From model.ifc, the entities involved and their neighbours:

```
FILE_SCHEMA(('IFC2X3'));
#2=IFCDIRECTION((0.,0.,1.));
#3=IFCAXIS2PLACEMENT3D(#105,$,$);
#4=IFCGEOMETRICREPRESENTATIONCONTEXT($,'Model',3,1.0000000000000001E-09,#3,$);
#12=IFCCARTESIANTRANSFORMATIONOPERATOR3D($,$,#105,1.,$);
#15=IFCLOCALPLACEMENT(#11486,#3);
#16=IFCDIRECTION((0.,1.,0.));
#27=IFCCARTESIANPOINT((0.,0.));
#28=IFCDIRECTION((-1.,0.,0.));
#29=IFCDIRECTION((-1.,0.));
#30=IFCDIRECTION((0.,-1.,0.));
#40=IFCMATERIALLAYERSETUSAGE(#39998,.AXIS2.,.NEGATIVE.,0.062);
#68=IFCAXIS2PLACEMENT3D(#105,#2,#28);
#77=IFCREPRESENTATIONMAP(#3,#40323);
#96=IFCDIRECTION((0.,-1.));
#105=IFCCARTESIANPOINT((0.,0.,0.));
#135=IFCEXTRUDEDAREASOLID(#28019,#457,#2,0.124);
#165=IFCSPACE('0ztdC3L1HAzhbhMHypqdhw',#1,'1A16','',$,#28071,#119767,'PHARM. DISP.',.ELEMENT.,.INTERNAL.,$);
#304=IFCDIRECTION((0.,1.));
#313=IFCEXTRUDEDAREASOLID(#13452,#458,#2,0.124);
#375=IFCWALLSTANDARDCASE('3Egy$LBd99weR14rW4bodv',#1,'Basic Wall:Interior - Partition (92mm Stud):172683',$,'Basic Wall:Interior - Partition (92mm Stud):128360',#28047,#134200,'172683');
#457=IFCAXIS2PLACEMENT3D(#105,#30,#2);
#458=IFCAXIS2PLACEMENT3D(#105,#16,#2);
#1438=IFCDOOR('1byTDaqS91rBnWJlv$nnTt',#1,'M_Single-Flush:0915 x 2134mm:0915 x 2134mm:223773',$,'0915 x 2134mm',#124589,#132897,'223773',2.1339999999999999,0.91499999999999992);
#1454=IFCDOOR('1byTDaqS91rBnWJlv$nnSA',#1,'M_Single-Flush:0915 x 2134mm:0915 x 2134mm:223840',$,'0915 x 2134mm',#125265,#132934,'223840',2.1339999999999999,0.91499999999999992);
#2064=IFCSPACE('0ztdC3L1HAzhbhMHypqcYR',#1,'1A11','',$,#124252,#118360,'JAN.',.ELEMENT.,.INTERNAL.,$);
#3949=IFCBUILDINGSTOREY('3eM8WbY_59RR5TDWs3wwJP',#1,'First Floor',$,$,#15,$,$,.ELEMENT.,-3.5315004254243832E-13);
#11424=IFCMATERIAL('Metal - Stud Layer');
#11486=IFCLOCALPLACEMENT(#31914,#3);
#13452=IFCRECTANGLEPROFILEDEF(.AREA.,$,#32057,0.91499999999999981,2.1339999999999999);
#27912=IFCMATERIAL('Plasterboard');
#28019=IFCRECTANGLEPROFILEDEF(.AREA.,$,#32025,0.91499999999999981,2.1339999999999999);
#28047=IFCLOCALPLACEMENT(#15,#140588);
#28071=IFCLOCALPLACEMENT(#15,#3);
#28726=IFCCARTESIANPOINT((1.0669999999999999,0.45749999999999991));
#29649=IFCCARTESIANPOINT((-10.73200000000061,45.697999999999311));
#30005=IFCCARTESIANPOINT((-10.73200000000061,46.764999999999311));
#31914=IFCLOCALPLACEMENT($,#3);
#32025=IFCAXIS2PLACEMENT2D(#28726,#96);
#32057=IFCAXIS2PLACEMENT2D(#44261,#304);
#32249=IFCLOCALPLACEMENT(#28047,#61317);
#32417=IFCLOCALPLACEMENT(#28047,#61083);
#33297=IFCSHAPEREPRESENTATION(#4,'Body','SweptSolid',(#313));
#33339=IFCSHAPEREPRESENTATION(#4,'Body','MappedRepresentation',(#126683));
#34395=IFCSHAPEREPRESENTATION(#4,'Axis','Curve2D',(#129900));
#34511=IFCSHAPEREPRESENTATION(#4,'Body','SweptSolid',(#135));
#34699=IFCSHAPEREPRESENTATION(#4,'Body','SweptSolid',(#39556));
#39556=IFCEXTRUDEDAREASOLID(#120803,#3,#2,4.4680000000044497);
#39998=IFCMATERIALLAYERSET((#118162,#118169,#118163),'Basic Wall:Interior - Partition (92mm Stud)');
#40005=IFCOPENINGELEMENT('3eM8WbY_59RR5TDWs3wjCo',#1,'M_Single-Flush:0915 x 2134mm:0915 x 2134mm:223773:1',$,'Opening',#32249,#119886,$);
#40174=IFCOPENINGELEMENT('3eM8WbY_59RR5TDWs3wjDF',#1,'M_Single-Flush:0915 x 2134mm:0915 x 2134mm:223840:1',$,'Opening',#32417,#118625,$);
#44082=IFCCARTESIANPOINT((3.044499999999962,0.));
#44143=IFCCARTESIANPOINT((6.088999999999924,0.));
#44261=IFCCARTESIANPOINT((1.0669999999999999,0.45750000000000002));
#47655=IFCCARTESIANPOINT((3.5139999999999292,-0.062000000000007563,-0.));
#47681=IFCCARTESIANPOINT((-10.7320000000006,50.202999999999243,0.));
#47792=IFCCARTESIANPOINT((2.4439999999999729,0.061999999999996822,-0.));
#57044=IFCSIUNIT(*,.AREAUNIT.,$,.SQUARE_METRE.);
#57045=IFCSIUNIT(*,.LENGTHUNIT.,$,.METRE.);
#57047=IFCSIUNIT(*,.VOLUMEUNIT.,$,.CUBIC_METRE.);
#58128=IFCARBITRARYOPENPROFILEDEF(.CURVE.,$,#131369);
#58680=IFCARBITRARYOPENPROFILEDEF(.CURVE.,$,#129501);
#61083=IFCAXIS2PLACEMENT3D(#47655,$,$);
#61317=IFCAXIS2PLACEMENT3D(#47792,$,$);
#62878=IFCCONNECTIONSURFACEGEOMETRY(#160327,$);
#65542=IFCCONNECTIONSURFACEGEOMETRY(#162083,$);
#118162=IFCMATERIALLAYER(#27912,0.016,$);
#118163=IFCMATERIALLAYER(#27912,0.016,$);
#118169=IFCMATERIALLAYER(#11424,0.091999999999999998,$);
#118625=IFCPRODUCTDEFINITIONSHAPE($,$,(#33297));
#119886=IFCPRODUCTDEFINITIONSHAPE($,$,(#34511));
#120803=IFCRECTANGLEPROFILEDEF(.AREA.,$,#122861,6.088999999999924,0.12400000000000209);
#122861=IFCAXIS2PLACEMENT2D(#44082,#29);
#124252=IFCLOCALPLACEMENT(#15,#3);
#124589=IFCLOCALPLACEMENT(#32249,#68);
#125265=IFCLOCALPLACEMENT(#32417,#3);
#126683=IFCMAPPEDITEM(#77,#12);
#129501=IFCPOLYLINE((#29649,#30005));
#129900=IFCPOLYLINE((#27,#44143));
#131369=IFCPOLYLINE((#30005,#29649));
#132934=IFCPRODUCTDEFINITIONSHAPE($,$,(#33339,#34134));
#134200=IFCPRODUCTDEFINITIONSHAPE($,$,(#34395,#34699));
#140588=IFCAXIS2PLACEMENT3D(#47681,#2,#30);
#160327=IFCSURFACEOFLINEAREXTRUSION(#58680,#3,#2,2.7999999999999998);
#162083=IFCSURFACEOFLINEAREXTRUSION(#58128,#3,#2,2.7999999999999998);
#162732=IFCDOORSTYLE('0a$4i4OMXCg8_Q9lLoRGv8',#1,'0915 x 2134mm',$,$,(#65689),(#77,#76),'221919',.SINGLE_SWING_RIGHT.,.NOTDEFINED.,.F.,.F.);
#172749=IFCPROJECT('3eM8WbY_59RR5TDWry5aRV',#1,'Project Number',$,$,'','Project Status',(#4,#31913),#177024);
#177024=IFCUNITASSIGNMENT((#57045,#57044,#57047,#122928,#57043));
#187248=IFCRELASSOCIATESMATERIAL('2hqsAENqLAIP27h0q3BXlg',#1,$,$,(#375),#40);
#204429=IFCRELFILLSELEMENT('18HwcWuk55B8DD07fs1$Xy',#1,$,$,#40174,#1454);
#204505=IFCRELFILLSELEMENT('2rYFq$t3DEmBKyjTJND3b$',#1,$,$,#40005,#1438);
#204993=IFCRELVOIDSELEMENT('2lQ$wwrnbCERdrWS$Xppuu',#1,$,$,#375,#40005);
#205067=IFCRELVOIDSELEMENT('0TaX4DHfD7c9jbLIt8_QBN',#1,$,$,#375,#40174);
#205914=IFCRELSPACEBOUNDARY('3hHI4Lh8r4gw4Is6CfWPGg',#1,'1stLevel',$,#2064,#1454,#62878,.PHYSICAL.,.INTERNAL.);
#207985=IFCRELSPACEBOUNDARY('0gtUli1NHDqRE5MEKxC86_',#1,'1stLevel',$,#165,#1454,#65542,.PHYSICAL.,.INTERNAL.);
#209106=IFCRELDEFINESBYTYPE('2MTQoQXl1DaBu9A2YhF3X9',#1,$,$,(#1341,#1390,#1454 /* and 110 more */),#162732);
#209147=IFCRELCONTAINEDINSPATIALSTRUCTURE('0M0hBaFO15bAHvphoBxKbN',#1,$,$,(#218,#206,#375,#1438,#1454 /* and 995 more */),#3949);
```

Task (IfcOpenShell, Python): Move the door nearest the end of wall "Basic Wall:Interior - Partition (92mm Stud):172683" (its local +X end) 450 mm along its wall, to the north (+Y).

```python
import numpy as np
import ifcopenshell
import ifcopenshell.api.geometry
import ifcopenshell.util.placement
import ifcopenshell.util.unit

model = ifcopenshell.open("model.ifc")
unit_scale = ifcopenshell.util.unit.calculate_unit_scale(model)

door = model.by_guid("1byTDaqS91rBnWJlv$nnSA")
opening = door.FillsVoids[0].RelatingOpeningElement
wall = opening.VoidsElements[0].RelatingBuildingElement

wall_matrix = ifcopenshell.util.placement.get_local_placement(wall.ObjectPlacement)
shift = wall_matrix[:3, 0] * -0.45 / unit_scale
before = ifcopenshell.util.placement.get_local_placement(door.ObjectPlacement)[:3, 3].copy()

# The door is placed relative to its opening, so it follows when the opening moves.
matrix = ifcopenshell.util.placement.get_local_placement(opening.ObjectPlacement)
matrix[:3, 3] += shift
ifcopenshell.api.geometry.edit_object_placement(
    model, product=opening, matrix=matrix, is_si=False, should_transform_children=True
)

# Space boundary surfaces are stored in each space's coordinates; move them too.
for rel in door.ProvidesBoundaries:
    if not rel.ConnectionGeometry:
        continue
    surface = rel.ConnectionGeometry.SurfaceOnRelatingElement
    space_matrix = ifcopenshell.util.placement.get_local_placement(rel.RelatingSpace.ObjectPlacement)
    point = np.array(surface.Position.Location.Coordinates) + space_matrix[:3, :3].T @ shift
    surface.Position = model.createIfcAxis2Placement3D(
        model.createIfcCartesianPoint(point.tolist()), surface.Position.Axis, surface.Position.RefDirection
    )

after = ifcopenshell.util.placement.get_local_placement(door.ObjectPlacement)[:3, 3]
print("door moved by", (after - before).round(3) + 0.0)

model.write("model_edited.ifc")
```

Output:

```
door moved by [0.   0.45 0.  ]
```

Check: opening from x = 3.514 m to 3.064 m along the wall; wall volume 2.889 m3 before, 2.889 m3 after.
